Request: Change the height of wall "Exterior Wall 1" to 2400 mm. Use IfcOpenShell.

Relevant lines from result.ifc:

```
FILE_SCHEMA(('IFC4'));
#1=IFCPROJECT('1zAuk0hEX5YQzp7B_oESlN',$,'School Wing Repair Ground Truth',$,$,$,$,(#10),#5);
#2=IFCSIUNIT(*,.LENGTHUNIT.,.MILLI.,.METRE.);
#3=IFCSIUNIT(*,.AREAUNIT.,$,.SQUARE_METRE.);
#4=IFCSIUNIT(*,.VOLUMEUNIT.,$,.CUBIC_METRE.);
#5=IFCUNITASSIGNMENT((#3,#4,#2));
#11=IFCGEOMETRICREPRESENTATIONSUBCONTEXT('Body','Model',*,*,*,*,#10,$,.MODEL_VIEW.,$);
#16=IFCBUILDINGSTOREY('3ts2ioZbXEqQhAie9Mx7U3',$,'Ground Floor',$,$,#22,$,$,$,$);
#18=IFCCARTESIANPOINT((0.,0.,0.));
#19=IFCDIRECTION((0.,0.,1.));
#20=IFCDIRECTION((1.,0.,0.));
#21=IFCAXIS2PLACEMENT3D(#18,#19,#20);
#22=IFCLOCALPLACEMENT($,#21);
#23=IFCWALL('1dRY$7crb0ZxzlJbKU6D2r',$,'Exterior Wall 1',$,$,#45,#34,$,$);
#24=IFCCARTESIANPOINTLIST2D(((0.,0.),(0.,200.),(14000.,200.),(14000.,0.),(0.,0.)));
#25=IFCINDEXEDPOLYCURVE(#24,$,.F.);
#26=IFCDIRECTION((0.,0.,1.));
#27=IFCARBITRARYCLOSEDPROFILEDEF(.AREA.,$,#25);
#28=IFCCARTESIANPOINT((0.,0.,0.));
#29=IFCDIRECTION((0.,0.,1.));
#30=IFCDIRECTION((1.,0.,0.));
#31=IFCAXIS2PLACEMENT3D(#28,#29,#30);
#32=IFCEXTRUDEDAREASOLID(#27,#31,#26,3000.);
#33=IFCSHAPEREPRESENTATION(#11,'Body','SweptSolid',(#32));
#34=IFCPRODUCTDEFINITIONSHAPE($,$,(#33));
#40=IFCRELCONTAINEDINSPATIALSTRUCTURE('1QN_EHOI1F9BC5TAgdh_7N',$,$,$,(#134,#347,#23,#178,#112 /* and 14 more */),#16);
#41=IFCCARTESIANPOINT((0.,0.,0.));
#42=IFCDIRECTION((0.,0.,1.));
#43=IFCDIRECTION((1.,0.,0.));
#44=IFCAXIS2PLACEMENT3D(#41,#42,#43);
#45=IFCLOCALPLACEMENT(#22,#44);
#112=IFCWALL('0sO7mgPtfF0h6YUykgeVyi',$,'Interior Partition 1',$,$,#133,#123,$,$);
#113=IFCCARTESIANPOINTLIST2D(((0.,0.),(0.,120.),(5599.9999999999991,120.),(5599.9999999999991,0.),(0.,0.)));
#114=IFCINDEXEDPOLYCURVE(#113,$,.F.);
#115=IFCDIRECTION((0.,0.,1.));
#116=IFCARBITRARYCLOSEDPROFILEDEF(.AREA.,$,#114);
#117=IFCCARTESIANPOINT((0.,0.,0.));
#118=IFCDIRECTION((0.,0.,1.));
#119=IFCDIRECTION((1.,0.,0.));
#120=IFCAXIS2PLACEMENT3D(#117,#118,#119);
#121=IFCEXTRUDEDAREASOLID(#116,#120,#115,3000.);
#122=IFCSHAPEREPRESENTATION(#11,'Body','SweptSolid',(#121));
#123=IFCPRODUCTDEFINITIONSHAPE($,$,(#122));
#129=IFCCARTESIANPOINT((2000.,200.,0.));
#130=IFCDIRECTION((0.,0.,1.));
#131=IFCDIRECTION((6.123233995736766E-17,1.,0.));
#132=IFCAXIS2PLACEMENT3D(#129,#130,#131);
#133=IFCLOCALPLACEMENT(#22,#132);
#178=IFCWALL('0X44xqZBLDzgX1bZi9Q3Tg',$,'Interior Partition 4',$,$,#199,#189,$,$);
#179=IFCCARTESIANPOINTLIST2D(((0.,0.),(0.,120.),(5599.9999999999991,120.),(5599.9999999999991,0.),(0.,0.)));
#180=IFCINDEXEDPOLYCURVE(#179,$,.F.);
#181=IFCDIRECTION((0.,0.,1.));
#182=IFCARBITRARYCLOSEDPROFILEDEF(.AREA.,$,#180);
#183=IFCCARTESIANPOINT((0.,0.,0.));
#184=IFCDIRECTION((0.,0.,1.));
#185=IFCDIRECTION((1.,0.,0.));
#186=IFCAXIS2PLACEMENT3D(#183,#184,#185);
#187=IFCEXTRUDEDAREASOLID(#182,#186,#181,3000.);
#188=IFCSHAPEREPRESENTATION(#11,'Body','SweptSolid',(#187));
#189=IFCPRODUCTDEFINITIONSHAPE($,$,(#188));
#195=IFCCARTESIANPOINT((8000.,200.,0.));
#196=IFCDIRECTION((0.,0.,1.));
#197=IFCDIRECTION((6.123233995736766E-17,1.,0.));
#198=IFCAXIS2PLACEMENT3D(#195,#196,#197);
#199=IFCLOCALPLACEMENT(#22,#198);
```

```python
import ifcopenshell
import ifcopenshell.geom
import ifcopenshell.util.representation
import ifcopenshell.util.shape

model = ifcopenshell.open("result.ifc")
settings = ifcopenshell.geom.settings()


def volume(element):
    """Net volume in cubic metres, openings subtracted."""
    shape = ifcopenshell.geom.create_shape(settings, element)
    return ifcopenshell.util.shape.get_volume(shape.geometry)


wall = model.by_guid("1dRY$7crb0ZxzlJbKU6D2r")
before = volume(wall)

body = ifcopenshell.util.representation.get_representation(wall, "Model", "Body")
solid = body.Items[0]
old_height = solid.Depth
solid.Depth = 2400.0
after = volume(wall)

print(f"height {old_height:g} -> {solid.Depth:g}, volume {before:.3f} -> {after:.3f} m3")

model.write("result_rev.ifc")
```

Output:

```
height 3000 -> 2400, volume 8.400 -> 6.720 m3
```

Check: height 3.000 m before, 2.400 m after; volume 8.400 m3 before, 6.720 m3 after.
